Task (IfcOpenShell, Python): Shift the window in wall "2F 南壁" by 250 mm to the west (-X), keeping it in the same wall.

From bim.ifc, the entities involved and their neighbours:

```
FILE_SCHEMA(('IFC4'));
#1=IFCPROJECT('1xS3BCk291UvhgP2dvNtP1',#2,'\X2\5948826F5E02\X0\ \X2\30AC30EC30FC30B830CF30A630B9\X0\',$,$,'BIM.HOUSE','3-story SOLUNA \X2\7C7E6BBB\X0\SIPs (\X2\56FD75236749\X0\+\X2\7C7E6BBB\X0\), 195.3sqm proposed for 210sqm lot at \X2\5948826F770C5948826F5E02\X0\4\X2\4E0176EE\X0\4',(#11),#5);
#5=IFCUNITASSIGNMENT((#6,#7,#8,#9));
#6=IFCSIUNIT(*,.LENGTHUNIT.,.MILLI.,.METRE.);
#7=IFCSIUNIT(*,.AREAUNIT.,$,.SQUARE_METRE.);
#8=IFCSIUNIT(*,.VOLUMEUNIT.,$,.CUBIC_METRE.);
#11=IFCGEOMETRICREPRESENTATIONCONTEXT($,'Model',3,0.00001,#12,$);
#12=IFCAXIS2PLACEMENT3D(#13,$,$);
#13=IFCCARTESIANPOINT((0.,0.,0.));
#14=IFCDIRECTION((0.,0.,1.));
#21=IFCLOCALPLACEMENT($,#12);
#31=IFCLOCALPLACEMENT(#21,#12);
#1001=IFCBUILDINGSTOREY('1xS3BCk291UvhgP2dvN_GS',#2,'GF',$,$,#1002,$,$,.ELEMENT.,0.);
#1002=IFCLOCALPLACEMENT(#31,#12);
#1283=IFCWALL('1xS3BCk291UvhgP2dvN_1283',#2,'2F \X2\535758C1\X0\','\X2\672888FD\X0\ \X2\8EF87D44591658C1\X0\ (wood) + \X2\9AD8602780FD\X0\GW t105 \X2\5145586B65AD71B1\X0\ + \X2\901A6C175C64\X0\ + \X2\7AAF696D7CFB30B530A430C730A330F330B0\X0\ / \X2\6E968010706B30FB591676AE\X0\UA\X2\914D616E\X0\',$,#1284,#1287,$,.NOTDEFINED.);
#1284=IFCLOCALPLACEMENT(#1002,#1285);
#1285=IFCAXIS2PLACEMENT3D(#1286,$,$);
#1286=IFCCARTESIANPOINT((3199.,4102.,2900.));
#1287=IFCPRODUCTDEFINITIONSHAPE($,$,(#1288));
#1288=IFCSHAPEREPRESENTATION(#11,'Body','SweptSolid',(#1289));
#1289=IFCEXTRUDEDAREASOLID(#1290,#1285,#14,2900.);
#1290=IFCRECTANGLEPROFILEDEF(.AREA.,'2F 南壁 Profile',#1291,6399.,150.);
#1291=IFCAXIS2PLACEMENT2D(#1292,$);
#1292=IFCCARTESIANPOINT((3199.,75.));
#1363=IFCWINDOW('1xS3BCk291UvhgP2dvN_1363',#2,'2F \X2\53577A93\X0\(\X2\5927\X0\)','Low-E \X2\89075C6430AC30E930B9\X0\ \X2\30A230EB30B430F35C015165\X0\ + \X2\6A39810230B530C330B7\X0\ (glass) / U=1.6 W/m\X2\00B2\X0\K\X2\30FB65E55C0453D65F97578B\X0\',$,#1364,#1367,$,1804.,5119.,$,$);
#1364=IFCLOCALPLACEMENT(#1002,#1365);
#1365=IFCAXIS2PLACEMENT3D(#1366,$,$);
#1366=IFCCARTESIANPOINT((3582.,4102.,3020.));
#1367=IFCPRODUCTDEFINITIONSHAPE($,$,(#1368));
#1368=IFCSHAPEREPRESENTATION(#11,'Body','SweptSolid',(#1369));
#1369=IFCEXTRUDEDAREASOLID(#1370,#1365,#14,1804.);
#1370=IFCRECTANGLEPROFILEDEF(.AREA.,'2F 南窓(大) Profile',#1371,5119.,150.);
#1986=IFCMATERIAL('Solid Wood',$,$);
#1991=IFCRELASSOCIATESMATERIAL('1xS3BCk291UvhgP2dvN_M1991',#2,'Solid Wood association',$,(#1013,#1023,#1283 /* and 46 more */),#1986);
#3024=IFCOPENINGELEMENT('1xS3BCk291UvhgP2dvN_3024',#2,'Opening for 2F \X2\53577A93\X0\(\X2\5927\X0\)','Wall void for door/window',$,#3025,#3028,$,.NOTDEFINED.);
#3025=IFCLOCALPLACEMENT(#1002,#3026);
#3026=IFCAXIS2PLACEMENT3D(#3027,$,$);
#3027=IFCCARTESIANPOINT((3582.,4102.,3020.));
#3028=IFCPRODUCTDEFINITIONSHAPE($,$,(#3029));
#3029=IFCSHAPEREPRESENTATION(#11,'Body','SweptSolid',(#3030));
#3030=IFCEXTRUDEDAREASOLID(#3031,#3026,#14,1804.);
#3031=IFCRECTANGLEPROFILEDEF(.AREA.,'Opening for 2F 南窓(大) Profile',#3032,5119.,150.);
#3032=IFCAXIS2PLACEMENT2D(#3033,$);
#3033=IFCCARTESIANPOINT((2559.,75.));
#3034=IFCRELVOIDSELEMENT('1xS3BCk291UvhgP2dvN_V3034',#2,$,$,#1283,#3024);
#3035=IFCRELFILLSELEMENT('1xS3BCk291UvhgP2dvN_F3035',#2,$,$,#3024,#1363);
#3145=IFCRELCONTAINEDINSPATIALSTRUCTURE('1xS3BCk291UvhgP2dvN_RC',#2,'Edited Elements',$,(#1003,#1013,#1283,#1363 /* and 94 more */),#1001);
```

```python
import ifcopenshell
import ifcopenshell.api.geometry
import ifcopenshell.util.placement
import ifcopenshell.util.unit

model = ifcopenshell.open("bim.ifc")
unit_scale = ifcopenshell.util.unit.calculate_unit_scale(model)

window = model.by_guid("1xS3BCk291UvhgP2dvN_1363")
opening = window.FillsVoids[0].RelatingOpeningElement
wall = opening.VoidsElements[0].RelatingBuildingElement

wall_matrix = ifcopenshell.util.placement.get_local_placement(wall.ObjectPlacement)
shift = wall_matrix[:3, 0] * -0.25 / unit_scale
before = ifcopenshell.util.placement.get_local_placement(window.ObjectPlacement)[:3, 3].copy()

# The window is not placed relative to its opening, so move both.
for product in (opening, window):
    matrix = ifcopenshell.util.placement.get_local_placement(product.ObjectPlacement)
    matrix[:3, 3] += shift
    ifcopenshell.api.geometry.edit_object_placement(model, product=product, matrix=matrix, is_si=False)

after = ifcopenshell.util.placement.get_local_placement(window.ObjectPlacement)[:3, 3]
print("window moved by", (after - before).round(3) + 0.0)

model.write("bim_v2.ifc")
```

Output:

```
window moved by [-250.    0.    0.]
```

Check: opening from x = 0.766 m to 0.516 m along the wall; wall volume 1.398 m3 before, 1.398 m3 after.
